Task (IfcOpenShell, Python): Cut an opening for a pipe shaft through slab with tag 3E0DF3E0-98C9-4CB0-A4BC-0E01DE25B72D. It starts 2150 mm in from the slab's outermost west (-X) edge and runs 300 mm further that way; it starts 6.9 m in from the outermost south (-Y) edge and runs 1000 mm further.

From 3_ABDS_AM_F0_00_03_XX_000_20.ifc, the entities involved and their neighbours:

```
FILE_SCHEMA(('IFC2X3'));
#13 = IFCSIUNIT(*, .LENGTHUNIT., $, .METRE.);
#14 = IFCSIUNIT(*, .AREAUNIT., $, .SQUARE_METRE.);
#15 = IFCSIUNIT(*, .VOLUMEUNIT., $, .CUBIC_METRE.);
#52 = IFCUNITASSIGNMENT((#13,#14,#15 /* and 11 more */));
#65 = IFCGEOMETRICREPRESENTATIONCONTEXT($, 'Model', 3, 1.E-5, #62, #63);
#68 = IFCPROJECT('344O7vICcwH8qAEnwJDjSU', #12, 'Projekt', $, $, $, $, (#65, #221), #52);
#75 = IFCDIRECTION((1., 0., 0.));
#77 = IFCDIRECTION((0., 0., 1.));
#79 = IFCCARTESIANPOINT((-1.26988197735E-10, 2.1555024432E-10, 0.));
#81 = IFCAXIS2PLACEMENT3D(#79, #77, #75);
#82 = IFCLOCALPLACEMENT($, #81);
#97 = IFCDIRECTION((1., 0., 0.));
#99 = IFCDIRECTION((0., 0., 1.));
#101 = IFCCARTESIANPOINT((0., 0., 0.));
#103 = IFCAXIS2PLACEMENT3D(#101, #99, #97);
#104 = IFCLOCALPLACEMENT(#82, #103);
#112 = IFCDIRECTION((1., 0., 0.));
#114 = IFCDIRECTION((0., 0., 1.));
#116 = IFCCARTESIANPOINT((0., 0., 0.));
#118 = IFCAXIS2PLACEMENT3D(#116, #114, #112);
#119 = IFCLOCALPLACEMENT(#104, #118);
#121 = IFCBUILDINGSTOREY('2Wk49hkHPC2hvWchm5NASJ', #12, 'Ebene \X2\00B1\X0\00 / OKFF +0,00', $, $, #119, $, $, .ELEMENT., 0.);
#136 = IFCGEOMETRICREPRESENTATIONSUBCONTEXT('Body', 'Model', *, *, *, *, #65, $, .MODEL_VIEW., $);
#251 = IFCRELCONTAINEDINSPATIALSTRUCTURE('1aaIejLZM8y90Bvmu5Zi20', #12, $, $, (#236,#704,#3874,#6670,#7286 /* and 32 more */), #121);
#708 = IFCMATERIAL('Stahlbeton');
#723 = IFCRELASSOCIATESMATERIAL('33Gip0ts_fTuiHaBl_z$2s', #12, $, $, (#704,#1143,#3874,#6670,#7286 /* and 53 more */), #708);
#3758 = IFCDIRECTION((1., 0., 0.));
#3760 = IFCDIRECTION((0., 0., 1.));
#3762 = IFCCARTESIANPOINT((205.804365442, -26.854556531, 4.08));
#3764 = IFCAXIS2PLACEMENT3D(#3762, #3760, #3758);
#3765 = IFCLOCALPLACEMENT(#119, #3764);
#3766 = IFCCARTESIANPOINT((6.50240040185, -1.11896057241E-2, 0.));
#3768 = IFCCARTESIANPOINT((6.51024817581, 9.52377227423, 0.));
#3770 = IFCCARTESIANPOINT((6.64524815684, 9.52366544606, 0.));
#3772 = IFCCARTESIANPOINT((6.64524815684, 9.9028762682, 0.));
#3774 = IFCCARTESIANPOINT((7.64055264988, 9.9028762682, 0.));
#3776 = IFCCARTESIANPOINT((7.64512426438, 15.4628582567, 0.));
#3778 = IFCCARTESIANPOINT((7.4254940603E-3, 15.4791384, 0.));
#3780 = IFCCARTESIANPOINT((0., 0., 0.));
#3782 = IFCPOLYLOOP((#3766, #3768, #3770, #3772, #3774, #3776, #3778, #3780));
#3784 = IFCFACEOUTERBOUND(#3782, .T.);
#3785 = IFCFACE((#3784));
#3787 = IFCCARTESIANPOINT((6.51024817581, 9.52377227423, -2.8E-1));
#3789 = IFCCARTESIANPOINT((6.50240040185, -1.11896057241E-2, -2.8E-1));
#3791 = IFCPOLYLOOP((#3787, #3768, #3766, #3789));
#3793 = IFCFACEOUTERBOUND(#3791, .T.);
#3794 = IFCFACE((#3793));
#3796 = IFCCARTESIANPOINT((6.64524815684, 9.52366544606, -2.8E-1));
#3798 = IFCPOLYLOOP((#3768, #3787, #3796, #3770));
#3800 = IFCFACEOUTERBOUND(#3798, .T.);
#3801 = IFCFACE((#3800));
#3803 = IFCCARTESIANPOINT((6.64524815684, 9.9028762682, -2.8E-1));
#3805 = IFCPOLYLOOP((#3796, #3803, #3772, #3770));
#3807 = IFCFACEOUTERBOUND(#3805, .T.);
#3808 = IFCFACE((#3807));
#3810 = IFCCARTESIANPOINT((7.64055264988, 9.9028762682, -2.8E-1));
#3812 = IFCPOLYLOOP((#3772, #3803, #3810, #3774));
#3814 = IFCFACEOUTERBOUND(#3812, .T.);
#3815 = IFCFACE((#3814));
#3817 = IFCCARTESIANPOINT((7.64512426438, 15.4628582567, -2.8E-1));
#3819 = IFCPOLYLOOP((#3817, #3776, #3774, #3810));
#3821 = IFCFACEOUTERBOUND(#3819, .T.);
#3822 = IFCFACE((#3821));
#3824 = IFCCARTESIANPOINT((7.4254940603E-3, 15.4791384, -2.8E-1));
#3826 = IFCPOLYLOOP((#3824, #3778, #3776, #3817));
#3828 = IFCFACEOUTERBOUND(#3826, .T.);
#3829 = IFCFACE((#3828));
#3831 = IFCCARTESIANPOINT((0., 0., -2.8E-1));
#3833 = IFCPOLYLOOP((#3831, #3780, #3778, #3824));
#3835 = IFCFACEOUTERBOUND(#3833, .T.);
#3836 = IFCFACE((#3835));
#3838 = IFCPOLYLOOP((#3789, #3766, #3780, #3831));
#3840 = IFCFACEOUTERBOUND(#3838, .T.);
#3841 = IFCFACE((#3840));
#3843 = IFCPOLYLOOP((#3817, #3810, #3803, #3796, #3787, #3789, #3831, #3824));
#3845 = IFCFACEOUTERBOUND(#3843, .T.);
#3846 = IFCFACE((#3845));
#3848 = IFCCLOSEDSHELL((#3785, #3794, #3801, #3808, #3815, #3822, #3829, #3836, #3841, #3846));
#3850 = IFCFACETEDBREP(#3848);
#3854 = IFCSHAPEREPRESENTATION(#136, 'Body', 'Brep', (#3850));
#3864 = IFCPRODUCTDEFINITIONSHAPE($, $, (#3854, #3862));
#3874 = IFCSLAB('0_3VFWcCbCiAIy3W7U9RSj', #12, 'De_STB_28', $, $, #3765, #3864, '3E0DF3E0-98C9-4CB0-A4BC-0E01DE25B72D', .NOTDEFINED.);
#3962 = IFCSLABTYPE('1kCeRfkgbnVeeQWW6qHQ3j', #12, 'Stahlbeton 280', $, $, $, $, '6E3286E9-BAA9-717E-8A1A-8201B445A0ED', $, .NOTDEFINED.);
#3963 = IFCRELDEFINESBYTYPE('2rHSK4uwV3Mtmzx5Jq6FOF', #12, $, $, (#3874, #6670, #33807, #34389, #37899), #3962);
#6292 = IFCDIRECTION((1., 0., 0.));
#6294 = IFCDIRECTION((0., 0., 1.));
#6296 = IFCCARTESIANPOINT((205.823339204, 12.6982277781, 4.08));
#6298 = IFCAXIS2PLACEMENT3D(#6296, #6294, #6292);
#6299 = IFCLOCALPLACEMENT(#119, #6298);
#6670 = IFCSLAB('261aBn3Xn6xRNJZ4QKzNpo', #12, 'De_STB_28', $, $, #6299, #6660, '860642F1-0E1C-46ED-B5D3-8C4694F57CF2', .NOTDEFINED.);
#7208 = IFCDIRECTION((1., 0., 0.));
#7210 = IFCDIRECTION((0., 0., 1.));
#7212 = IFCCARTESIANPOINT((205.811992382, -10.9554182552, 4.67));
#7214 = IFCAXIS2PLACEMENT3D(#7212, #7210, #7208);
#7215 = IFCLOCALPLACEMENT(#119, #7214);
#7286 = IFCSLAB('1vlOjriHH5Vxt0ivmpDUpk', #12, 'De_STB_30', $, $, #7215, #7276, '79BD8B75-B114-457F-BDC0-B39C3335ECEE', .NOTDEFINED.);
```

```python
import numpy as np
import ifcopenshell
import ifcopenshell.api.feature
import ifcopenshell.api.geometry
import ifcopenshell.api.root
import ifcopenshell.geom
import ifcopenshell.util.placement
import ifcopenshell.util.representation
import ifcopenshell.util.shape
import ifcopenshell.util.unit

model = ifcopenshell.open("3_ABDS_AM_F0_00_03_XX_000_20.ifc")
unit_scale = ifcopenshell.util.unit.calculate_unit_scale(model)
settings = ifcopenshell.geom.settings()


def volume(element):
    """Net volume in cubic metres, openings subtracted."""
    shape = ifcopenshell.geom.create_shape(settings, element)
    return ifcopenshell.util.shape.get_volume(shape.geometry)


slab = model.by_guid("0_3VFWcCbCiAIy3W7U9RSj")
before = volume(slab)

# Extent in the slab's own axes, in metres. The edges named are its -X and -Y sides.
slab_shape = ifcopenshell.geom.create_shape(settings, slab)
vertices = ifcopenshell.util.shape.get_vertices(slab_shape.geometry)
x_min, y_min, bottom = vertices.min(axis=0)
top = vertices[:, 2].max()

opening = ifcopenshell.api.root.create_entity(model, ifc_class="IfcOpeningElement", name="Pipe shaft opening")
context = ifcopenshell.util.representation.get_context(model, "Model", "Body", "MODEL_VIEW")
width, depth = 0.3, 1
outline = [(0.0, 0.0), (width, 0.0), (width, depth), (0.0, depth), (0.0, 0.0)]
# Overshoot both faces by 50 mm so the cut is clean.
shape = ifcopenshell.api.geometry.add_slab_representation(
    model, context=context, depth=top - bottom + 0.1, polyline=outline
)
ifcopenshell.api.geometry.assign_representation(model, product=opening, representation=shape)

matrix = ifcopenshell.util.placement.get_local_placement(slab.ObjectPlacement)
matrix[:, 3] = matrix @ np.append(np.array([x_min + 2.15, y_min + 6.9, bottom - 0.05]) / unit_scale, 1.0)
ifcopenshell.api.geometry.edit_object_placement(model, product=opening, matrix=matrix, is_si=False)
ifcopenshell.api.feature.add_feature(model, feature=opening, element=slab)

after = volume(slab)

print(f"slab volume {before:.3f} -> {after:.3f} m3")

model.write("3_ABDS_AM_F0_00_03_XX_000_20-out.ifc")
```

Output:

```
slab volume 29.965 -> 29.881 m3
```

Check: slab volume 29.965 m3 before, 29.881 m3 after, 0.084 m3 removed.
